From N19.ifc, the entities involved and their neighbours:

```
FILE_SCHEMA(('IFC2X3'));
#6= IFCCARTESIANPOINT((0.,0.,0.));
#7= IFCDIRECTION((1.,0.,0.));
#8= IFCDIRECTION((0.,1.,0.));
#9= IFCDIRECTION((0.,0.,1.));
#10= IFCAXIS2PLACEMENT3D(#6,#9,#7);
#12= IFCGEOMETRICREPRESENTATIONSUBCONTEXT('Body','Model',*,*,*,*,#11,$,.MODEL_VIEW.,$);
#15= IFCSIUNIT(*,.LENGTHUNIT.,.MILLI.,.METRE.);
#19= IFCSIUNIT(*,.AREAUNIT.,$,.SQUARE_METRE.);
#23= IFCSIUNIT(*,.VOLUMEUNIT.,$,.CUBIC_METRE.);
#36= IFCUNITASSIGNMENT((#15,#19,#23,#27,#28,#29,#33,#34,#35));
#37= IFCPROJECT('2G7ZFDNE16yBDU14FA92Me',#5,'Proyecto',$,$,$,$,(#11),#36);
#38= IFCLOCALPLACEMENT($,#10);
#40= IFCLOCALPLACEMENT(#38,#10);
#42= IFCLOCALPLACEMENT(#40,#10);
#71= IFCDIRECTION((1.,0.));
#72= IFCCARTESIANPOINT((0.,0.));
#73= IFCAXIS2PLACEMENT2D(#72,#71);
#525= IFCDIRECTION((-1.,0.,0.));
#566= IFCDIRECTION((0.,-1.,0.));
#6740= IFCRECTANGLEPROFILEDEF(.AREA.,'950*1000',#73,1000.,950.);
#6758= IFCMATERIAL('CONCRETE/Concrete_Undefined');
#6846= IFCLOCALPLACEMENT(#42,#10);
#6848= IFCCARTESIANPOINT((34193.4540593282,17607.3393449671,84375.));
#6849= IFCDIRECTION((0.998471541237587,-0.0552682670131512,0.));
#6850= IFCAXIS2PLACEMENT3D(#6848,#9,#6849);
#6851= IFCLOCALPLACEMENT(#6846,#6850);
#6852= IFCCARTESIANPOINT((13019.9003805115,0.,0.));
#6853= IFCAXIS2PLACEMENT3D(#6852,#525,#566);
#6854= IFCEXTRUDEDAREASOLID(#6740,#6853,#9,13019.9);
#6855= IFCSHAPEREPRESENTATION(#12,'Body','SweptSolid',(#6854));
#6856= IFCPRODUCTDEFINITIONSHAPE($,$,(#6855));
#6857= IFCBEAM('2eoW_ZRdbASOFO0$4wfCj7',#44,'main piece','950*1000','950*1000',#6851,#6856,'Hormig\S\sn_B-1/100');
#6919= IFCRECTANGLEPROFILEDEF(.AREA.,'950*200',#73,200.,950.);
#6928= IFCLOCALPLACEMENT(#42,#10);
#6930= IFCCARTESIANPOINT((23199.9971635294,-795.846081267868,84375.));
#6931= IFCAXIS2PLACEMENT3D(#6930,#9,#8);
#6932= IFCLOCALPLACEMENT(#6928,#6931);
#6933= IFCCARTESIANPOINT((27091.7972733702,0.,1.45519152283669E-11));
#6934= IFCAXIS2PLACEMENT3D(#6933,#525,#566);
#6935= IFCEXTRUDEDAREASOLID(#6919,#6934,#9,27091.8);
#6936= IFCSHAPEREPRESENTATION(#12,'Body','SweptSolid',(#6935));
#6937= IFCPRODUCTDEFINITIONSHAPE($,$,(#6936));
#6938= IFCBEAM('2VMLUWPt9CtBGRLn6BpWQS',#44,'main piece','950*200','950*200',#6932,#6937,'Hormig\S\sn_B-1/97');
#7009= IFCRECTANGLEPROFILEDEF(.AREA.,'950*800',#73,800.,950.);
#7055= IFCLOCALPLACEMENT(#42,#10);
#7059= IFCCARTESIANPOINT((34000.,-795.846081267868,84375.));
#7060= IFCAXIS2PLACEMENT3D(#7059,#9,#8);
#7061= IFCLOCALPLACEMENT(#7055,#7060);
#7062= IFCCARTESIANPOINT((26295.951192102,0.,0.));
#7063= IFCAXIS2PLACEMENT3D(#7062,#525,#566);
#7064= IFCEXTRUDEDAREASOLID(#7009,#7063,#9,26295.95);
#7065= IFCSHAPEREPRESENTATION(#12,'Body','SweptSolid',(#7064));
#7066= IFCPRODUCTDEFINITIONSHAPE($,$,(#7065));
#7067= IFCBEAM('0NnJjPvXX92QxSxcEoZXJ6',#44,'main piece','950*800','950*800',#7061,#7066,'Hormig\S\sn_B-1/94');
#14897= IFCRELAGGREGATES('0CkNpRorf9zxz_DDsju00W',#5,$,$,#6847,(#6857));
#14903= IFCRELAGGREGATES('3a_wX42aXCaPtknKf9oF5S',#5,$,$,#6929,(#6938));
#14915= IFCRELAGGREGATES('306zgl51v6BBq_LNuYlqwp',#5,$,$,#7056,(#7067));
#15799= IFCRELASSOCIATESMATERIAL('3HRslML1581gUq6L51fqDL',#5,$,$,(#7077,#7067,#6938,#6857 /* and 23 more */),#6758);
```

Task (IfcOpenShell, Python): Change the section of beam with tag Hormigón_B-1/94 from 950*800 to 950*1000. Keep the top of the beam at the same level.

```python
import ifcopenshell
import ifcopenshell.util.element
import ifcopenshell.util.representation

model = ifcopenshell.open("N19.ifc")

member = model.by_guid("0NnJjPvXX92QxSxcEoZXJ6")
source = next(p for p in model.by_type("IfcRectangleProfileDef") if p.ProfileName == "950*1000")

body = ifcopenshell.util.representation.get_representation(member, "Model", "Body")
solid = body.Items[0]
old_profile = solid.SweptArea

# Copy the section's sizes but keep this member's own profile position.
profile = ifcopenshell.util.element.copy(model, source)
# Profiles are centred, so shift by half the change in depth to hold the top.
shift = (old_profile.YDim - profile.YDim) / 2
x, y = old_profile.Position.Location.Coordinates
up = (0.0, 1.0)  # upwards, in the solid's own plane
location = model.createIfcCartesianPoint((x + up[0] * shift, y + up[1] * shift))
profile.Position = model.createIfcAxis2Placement2D(location, old_profile.Position.RefDirection)
solid.SweptArea = profile
if not model.get_total_inverses(old_profile):
    ifcopenshell.util.element.remove_deep2(model, old_profile)
member.Description = member.Description.replace("950*800", "950*1000")
member.ObjectType = member.ObjectType.replace("950*800", "950*1000")

print(solid.SweptArea)

model.write("N19_rev.ifc")
```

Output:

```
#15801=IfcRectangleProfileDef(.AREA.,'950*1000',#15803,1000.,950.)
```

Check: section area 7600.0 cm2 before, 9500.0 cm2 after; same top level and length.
